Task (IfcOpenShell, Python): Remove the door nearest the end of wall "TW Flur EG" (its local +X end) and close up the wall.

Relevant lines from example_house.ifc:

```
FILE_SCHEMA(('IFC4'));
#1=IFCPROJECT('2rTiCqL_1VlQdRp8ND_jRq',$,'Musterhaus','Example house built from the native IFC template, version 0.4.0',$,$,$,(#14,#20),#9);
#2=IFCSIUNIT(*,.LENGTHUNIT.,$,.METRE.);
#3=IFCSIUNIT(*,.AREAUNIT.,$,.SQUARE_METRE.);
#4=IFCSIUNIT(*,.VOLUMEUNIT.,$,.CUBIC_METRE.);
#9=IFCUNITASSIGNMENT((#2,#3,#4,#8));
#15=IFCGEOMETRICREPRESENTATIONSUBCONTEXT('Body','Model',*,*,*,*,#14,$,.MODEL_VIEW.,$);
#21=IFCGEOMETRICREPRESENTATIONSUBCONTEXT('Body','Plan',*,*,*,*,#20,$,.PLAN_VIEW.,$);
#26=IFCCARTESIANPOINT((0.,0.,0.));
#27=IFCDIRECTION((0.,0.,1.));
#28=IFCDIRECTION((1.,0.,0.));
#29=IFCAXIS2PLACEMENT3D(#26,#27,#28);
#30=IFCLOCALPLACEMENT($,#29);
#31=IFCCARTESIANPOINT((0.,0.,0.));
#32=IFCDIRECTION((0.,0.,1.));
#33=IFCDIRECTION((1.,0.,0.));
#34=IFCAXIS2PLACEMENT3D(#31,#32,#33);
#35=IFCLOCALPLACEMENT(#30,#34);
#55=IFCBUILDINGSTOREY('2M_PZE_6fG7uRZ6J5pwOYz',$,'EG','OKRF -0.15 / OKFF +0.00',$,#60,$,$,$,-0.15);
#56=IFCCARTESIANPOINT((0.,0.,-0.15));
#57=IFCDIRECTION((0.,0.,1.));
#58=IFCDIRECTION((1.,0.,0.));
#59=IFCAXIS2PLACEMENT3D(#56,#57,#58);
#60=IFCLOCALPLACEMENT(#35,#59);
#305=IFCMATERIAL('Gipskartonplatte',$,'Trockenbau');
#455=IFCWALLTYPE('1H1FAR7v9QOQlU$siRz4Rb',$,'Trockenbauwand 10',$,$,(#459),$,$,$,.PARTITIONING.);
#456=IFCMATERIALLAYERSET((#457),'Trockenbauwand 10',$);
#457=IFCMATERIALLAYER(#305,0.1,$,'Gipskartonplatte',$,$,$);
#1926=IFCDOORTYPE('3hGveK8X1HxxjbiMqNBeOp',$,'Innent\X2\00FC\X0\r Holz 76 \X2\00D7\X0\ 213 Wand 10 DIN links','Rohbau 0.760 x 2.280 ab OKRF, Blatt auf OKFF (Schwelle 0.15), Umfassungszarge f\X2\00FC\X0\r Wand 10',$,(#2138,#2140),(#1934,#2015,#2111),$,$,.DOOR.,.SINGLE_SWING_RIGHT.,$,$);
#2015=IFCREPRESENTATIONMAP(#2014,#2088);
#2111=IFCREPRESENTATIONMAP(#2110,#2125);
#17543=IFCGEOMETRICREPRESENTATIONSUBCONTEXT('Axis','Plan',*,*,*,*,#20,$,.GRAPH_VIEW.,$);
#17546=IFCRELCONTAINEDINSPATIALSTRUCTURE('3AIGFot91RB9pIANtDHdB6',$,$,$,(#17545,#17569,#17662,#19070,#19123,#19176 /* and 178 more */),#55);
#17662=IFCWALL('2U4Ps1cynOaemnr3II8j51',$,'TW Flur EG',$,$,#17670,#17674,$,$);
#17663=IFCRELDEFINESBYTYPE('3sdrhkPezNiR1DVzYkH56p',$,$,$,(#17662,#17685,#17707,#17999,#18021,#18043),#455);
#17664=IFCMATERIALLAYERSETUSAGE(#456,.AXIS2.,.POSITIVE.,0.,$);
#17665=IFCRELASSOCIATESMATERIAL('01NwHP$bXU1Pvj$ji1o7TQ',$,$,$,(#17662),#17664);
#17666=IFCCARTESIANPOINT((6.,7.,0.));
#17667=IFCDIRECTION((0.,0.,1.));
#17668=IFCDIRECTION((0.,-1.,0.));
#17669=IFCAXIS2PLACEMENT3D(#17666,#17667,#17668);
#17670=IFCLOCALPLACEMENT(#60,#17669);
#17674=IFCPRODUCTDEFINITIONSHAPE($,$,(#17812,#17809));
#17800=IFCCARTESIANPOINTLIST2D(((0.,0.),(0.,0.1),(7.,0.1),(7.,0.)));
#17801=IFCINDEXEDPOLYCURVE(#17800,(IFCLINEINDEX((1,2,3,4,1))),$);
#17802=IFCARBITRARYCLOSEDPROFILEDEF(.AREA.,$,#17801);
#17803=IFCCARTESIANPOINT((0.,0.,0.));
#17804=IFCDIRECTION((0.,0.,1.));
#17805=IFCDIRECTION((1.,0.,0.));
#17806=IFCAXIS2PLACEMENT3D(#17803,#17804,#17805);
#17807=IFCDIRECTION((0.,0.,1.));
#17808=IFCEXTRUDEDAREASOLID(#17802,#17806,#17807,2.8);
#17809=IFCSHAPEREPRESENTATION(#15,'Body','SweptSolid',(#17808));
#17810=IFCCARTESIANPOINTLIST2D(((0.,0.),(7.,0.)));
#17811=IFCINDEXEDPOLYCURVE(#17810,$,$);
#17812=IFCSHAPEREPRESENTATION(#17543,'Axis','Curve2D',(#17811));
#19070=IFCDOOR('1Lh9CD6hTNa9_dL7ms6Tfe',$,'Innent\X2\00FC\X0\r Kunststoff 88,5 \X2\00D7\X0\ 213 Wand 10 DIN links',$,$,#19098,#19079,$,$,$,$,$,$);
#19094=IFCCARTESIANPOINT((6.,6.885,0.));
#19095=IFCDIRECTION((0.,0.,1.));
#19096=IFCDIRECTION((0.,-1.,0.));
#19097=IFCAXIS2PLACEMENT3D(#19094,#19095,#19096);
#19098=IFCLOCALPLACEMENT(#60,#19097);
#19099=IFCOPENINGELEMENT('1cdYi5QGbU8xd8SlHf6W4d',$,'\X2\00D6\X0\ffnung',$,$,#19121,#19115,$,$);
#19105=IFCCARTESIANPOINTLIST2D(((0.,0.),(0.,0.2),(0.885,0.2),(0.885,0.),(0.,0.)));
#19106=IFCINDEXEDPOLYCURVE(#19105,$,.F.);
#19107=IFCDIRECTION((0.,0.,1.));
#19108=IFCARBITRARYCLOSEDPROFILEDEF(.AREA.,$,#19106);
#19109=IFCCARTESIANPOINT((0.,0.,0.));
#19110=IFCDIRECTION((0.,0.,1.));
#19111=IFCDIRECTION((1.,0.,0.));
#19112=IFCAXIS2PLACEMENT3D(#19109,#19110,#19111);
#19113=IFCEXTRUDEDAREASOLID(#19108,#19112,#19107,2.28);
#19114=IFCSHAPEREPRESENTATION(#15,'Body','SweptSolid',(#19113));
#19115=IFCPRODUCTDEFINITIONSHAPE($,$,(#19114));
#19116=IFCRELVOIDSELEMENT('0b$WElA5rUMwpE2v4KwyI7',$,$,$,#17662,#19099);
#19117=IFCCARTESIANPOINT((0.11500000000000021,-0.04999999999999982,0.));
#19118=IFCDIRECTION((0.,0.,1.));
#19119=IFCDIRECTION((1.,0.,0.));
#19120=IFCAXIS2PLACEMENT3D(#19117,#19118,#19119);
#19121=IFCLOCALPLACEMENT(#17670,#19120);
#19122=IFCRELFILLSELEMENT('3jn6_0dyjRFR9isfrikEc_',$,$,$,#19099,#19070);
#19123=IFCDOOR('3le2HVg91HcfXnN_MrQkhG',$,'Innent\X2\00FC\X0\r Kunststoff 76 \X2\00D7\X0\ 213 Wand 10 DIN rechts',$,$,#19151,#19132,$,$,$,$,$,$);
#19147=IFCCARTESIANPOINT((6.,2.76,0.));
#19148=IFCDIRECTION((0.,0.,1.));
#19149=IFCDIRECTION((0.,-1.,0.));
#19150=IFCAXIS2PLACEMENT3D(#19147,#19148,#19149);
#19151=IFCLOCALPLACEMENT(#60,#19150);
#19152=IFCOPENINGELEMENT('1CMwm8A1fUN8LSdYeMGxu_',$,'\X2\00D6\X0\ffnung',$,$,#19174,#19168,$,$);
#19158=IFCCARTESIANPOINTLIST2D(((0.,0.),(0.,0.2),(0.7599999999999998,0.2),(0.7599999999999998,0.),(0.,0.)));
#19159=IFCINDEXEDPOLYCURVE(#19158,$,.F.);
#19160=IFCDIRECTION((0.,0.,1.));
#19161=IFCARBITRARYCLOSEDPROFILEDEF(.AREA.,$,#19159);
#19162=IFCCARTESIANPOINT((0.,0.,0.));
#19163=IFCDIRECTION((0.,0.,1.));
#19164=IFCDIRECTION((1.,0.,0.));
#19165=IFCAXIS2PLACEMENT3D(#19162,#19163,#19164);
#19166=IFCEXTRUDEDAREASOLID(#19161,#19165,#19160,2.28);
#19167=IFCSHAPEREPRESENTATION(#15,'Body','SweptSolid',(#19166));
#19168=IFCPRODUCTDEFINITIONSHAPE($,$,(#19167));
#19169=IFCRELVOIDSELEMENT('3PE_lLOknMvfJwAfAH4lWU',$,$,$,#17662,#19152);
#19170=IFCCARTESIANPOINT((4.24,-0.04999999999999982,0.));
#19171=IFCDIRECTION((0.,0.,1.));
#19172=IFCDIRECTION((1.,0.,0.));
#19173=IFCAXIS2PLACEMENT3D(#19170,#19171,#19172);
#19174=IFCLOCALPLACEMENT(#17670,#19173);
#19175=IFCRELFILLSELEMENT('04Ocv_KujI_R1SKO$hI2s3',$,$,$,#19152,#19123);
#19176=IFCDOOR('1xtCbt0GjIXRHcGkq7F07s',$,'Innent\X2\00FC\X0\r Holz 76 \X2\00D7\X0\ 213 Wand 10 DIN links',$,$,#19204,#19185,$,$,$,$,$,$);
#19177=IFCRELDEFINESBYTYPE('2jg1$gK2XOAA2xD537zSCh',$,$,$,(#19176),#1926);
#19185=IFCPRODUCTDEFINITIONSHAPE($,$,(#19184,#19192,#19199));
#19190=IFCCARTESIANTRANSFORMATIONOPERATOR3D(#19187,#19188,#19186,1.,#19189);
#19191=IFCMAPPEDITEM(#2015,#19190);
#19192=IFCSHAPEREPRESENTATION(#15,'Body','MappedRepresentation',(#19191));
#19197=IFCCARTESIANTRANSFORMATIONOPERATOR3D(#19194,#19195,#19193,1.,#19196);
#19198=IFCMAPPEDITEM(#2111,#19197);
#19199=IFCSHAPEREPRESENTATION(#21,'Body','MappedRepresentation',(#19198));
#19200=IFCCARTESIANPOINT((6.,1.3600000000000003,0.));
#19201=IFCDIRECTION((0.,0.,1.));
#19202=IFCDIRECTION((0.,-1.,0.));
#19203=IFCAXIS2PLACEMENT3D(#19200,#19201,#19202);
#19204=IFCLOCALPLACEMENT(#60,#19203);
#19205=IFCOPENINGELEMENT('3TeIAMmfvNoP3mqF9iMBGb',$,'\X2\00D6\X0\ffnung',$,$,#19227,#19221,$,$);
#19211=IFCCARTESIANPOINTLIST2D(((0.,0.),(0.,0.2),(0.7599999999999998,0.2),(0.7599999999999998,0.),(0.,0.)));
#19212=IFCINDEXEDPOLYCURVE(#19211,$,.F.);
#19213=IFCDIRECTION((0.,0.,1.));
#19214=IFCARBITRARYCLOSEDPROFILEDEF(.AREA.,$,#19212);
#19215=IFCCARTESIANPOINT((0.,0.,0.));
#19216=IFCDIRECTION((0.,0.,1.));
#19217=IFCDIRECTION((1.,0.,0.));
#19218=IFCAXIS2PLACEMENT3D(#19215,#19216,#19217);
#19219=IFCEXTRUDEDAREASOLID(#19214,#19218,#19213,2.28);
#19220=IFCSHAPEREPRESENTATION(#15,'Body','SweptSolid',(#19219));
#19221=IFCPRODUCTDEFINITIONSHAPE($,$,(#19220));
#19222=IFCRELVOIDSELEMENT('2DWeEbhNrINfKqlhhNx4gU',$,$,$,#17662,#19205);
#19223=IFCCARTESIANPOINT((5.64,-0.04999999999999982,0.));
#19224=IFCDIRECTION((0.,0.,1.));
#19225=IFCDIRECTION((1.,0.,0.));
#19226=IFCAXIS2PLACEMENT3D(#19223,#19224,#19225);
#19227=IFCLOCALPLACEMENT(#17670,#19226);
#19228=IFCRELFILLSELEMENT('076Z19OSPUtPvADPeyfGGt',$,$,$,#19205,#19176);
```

```python
import ifcopenshell
import ifcopenshell.api.feature
import ifcopenshell.api.root
import ifcopenshell.geom
import ifcopenshell.util.shape

model = ifcopenshell.open("example_house.ifc")
settings = ifcopenshell.geom.settings()


def volume(element):
    """Net volume in cubic metres, openings subtracted."""
    shape = ifcopenshell.geom.create_shape(settings, element)
    return ifcopenshell.util.shape.get_volume(shape.geometry)


door = model.by_guid("1xtCbt0GjIXRHcGkq7F07s")
opening = door.FillsVoids[0].RelatingOpeningElement
wall = opening.VoidsElements[0].RelatingBuildingElement
before = volume(wall)

ifcopenshell.api.root.remove_product(model, product=door)
ifcopenshell.api.feature.remove_feature(model, feature=opening)

after = volume(wall)

print(f"wall volume {before:.3f} -> {after:.3f} m3")

model.write("example_house-out.ifc")
```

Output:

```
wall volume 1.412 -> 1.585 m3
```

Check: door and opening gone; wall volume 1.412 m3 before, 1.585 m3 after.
